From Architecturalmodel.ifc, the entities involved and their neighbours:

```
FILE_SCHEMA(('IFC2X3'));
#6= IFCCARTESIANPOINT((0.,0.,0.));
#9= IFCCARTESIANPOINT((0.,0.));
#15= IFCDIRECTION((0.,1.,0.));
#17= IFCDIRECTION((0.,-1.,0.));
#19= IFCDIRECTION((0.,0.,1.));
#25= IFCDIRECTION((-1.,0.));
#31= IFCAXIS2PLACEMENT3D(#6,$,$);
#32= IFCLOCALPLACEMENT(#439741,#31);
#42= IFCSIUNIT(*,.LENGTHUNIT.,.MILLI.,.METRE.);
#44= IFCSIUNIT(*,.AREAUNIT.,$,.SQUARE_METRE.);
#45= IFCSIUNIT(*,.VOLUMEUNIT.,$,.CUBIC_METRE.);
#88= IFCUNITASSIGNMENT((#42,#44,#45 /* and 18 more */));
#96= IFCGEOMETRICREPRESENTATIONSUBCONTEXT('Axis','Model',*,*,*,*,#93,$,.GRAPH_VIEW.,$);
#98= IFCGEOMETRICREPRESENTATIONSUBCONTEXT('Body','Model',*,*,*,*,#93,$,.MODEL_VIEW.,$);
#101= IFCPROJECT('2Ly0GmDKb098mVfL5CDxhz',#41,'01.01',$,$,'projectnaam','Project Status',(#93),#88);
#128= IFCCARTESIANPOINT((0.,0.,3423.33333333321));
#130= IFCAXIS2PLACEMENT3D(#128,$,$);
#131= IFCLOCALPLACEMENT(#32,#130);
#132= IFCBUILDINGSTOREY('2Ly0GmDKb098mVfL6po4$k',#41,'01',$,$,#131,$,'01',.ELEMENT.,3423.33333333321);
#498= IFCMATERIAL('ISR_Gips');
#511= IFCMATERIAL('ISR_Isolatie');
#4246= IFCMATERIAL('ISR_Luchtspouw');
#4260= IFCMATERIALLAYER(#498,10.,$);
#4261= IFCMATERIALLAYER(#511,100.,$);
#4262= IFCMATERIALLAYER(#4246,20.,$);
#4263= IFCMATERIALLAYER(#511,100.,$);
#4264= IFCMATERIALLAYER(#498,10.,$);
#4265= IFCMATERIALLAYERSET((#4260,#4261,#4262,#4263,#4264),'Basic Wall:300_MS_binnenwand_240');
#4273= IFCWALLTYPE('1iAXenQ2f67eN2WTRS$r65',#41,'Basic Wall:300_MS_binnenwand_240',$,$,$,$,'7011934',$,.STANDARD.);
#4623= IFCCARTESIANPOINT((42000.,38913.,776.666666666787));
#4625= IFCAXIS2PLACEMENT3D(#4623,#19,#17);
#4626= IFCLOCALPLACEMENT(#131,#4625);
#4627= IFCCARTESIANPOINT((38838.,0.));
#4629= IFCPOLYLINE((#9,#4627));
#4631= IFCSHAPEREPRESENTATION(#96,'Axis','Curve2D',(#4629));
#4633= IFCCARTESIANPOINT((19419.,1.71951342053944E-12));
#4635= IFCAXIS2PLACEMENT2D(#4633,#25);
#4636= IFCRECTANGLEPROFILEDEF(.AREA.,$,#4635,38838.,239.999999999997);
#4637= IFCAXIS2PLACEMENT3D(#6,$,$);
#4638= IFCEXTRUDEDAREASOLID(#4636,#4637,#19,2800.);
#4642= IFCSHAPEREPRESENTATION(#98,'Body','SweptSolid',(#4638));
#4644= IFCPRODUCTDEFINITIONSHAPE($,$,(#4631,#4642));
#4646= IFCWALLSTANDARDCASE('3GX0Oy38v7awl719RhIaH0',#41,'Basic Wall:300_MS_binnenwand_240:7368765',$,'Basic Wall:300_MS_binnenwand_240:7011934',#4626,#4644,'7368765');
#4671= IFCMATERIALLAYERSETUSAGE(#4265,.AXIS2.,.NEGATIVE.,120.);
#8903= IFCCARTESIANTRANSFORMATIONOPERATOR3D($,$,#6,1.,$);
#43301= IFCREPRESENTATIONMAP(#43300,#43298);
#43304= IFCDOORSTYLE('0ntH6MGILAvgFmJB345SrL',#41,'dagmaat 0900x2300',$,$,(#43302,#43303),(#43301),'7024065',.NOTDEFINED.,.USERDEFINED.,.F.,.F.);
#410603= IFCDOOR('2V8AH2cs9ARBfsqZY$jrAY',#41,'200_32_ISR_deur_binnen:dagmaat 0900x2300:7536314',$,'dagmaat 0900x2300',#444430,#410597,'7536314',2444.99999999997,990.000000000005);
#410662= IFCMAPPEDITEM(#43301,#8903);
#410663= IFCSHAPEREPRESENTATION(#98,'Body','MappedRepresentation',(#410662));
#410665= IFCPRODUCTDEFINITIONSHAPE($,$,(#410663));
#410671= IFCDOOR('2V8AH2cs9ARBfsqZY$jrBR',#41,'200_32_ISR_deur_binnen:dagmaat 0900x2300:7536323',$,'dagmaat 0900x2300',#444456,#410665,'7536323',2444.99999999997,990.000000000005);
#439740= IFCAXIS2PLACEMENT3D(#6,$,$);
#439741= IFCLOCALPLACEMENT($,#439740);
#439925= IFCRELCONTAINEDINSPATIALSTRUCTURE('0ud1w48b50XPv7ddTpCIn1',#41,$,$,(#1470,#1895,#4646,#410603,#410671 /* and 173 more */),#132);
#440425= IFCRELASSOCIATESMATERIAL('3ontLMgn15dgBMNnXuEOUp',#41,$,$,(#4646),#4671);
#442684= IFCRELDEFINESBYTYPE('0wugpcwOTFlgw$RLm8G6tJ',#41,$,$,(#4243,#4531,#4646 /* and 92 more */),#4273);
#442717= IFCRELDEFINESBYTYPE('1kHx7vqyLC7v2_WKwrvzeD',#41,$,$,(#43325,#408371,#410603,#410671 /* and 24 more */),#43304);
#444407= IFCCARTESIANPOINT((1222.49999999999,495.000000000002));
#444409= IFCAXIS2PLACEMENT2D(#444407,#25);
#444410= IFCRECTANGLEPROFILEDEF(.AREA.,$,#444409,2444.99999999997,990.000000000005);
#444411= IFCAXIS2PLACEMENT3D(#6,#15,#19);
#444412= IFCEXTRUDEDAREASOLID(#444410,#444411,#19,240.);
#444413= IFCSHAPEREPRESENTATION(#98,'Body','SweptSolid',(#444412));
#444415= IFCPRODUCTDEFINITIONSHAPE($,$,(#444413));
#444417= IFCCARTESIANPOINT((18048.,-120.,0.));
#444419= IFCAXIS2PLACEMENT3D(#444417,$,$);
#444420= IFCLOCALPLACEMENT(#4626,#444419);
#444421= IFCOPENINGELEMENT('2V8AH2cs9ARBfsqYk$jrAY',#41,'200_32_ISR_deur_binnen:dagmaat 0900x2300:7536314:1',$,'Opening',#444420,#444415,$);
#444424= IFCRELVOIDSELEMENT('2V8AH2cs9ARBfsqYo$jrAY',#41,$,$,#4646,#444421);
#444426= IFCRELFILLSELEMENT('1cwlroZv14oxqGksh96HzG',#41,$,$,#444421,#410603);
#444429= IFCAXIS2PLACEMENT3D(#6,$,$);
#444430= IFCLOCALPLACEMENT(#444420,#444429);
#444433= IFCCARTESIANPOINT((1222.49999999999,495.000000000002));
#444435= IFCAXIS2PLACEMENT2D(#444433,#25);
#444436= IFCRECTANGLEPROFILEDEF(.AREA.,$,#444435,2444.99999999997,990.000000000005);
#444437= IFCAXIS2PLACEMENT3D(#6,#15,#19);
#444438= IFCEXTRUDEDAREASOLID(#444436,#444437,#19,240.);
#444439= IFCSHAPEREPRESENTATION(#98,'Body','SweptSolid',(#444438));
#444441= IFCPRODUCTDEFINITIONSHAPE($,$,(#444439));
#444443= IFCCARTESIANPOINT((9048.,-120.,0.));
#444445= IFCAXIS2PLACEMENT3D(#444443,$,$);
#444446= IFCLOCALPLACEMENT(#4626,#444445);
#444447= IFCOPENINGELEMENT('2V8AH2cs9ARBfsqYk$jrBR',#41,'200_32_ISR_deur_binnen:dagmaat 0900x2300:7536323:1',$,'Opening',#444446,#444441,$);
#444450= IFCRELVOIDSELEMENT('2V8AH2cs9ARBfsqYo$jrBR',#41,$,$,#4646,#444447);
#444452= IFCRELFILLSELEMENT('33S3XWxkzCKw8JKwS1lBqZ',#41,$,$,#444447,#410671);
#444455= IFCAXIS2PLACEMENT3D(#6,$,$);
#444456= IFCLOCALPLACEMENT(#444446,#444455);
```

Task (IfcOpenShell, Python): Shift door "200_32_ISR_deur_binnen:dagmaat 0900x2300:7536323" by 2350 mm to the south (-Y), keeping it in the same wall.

```python
import ifcopenshell
import ifcopenshell.api.geometry
import ifcopenshell.util.placement

model = ifcopenshell.open("Architecturalmodel.ifc")

door = model.by_id(410671)
opening = door.FillsVoids[0].RelatingOpeningElement
wall = opening.VoidsElements[0].RelatingBuildingElement

wall_matrix = ifcopenshell.util.placement.get_local_placement(wall.ObjectPlacement)
shift = wall_matrix[:3, 0] * 2350.0
before = ifcopenshell.util.placement.get_local_placement(door.ObjectPlacement)[:3, 3].copy()

# The door is placed relative to its opening, so it follows when the opening moves.
matrix = ifcopenshell.util.placement.get_local_placement(opening.ObjectPlacement)
matrix[:3, 3] += shift
ifcopenshell.api.geometry.edit_object_placement(
    model, product=opening, matrix=matrix, is_si=False, should_transform_children=True
)

after = ifcopenshell.util.placement.get_local_placement(door.ObjectPlacement)[:3, 3]
print("door moved by", (after - before).round(3) + 0.0)

model.write("Architecturalmodel_v2.ifc")
```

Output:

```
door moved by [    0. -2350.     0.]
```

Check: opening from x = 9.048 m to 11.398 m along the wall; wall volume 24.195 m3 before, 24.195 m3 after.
